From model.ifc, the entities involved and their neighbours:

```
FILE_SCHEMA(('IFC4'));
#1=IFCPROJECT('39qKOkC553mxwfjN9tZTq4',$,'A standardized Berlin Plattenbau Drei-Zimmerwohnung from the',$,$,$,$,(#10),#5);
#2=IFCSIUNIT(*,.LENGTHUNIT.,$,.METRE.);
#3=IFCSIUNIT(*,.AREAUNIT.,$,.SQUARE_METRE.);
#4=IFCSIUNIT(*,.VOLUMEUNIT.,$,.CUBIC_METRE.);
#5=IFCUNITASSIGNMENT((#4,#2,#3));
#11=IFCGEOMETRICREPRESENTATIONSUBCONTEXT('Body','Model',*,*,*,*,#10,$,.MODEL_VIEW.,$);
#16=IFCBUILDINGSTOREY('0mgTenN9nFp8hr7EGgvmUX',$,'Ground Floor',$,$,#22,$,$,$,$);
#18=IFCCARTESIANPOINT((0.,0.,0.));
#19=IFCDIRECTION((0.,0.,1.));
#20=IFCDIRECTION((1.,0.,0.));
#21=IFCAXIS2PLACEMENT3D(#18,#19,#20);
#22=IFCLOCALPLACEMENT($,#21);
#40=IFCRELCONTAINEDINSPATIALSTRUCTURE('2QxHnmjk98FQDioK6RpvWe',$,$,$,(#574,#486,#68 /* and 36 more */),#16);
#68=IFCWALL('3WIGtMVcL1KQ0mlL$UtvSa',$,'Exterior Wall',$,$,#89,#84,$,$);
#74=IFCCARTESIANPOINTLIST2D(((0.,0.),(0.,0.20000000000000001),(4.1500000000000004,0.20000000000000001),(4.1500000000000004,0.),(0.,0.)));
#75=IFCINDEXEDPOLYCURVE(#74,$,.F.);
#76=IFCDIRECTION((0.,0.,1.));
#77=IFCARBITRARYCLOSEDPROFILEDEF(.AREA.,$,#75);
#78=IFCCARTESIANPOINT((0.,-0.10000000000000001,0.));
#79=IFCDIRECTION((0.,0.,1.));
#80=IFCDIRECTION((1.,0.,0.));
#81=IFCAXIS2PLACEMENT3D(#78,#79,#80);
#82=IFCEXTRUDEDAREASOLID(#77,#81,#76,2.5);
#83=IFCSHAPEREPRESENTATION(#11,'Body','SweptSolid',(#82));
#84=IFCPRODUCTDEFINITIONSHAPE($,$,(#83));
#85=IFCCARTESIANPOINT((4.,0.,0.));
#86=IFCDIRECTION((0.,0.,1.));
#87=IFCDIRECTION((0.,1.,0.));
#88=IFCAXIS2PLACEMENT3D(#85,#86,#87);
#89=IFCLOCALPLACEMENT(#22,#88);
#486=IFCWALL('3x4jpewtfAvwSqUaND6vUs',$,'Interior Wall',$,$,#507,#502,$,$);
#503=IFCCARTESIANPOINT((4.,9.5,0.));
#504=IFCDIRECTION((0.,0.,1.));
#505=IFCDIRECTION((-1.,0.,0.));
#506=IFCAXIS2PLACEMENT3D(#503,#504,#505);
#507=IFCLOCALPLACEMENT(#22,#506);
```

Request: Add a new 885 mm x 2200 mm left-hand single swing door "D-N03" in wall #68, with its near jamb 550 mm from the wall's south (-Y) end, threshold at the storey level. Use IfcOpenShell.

```python
import numpy as np
import ifcopenshell
import ifcopenshell.api.feature
import ifcopenshell.api.geometry
import ifcopenshell.api.root
import ifcopenshell.api.spatial
import ifcopenshell.geom
import ifcopenshell.util.element
import ifcopenshell.util.placement
import ifcopenshell.util.representation
import ifcopenshell.util.shape
import ifcopenshell.util.unit

model = ifcopenshell.open("model.ifc")
unit_scale = ifcopenshell.util.unit.calculate_unit_scale(model)
settings = ifcopenshell.geom.settings()


def volume(element):
    """Net volume in cubic metres, openings subtracted."""
    shape = ifcopenshell.geom.create_shape(settings, element)
    return ifcopenshell.util.shape.get_volume(shape.geometry)


wall = model.by_guid("3WIGtMVcL1KQ0mlL$UtvSa")
storey = ifcopenshell.util.element.get_container(wall, ifc_class="IfcBuildingStorey")
context = ifcopenshell.util.representation.get_context(model, "Model", "Body", "MODEL_VIEW")
before = volume(wall)

width, height, from_end, sill = 0.885, 2.2, 0.55, 0.0  # metres

# The wall runs along its own X axis, and the end named is its -X end.
wall_shape = ifcopenshell.geom.create_shape(settings, wall)
x, y, z = ifcopenshell.util.shape.get_vertices(wall_shape.geometry).T
start = x.min() + from_end
face, thickness = float(y.min()), float(y.max() - y.min())
wall_matrix = ifcopenshell.util.placement.get_local_placement(wall.ObjectPlacement)
level = ifcopenshell.util.placement.get_local_placement(storey.ObjectPlacement)[2, 3]


def in_wall(x, y):
    """Placement at x, y metres in the wall's axes, at sill height."""
    matrix = wall_matrix.copy()
    matrix[:, 3] = wall_matrix @ np.array([x / unit_scale, y / unit_scale, 0.0, 1.0])
    matrix[2, 3] = level + sill / unit_scale
    return matrix


# Opening: a box that overshoots both wall faces by 50 mm.
opening = ifcopenshell.api.root.create_entity(model, ifc_class="IfcOpeningElement", predefined_type="OPENING")
box = ifcopenshell.api.geometry.add_wall_representation(
    model, context=context, length=width, height=height, thickness=thickness + 0.1
)
ifcopenshell.api.geometry.assign_representation(model, product=opening, representation=box)
ifcopenshell.api.geometry.edit_object_placement(model, product=opening, matrix=in_wall(start, face - 0.05), is_si=False)
ifcopenshell.api.feature.add_feature(model, feature=opening, element=wall)

door = ifcopenshell.api.root.create_entity(model, ifc_class="IfcDoor", name="D-N03", predefined_type="DOOR")
door.OverallWidth, door.OverallHeight = width / unit_scale, height / unit_scale
door.OperationType = "SINGLE_SWING_LEFT"
body = ifcopenshell.api.geometry.add_door_representation(
    model,
    context=context,
    overall_width=door.OverallWidth,
    overall_height=door.OverallHeight,
    operation_type="SINGLE_SWING_LEFT",
    lining_properties={"LiningDepth": thickness / unit_scale, "ThresholdDepth": thickness / unit_scale},
)
ifcopenshell.api.geometry.assign_representation(model, product=door, representation=body)
ifcopenshell.api.spatial.assign_container(model, products=[door], relating_structure=storey)
ifcopenshell.api.feature.add_filling(model, opening=opening, element=door)

# The lining spans the wall, so the door starts at the wall face.
ifcopenshell.api.geometry.edit_object_placement(model, product=door, matrix=in_wall(start, face), is_si=False)

after = volume(wall)

print(f"wall volume {before:.3f} -> {after:.3f} m3")

model.write("model-out.ifc")
```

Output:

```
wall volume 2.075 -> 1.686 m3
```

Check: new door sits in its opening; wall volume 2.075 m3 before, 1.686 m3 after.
